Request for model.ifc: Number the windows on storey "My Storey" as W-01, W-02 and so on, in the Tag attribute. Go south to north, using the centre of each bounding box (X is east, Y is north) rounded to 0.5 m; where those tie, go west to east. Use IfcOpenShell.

First a look at what the model holds.

```python
import ifcopenshell
import ifcopenshell.util.element
import ifcopenshell.util.placement

model = ifcopenshell.open("model.ifc")
print(model.schema)
storey = next(s for s in model.by_type("IfcBuildingStorey") if s.Name == "My Storey")
windows = [e for e in ifcopenshell.util.element.get_decomposition(storey) if e.is_a("IfcWindow")]
for e in sorted(windows, key=lambda e: e.id()):
    origin = ifcopenshell.util.placement.get_local_placement(e.ObjectPlacement)[:3, 3]
    print(e.id(), e.Tag, e.Name, origin.round(2) + 0.0, sep=" | ")
```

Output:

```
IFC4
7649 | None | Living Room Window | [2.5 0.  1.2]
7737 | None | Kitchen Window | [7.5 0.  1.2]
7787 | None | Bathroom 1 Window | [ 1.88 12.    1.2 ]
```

```python
import ifcopenshell
import ifcopenshell.geom
import ifcopenshell.util.element
import ifcopenshell.util.shape

model = ifcopenshell.open("model.ifc")
settings = ifcopenshell.geom.settings()
settings.set("use-world-coords", True)


def centre(element):
    shape = ifcopenshell.geom.create_shape(settings, element)
    return ifcopenshell.util.shape.get_bbox_centroid(shape.geometry)


storey = next(s for s in model.by_type("IfcBuildingStorey") if s.Name == "My Storey")
windows = [e for e in ifcopenshell.util.element.get_decomposition(storey) if e.is_a("IfcWindow")]

# Insertion points can sit at a corner or the storey origin, so sort by the geometry (in metres).
centres = {e: centre(e) for e in windows}
windows.sort(key=lambda e: (round(centres[e][1] / 0.5), centres[e][0]))

for i, e in enumerate(windows, start=1):
    number = f"W-{i:02d}"
    e.Tag = number
    print(e.id(), number)

model.write("model_v2.ifc")
```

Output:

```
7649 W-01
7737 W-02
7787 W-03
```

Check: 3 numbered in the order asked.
